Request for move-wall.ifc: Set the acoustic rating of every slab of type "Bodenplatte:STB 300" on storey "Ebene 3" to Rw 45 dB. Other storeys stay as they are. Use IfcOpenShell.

First a look at what the model holds.

```python
import ifcopenshell
import ifcopenshell.util.element

model = ifcopenshell.open("move-wall.ifc")
print(model.schema)
storey = next(s for s in model.by_type("IfcBuildingStorey") if s.Name == "Ebene 3")
slabs = [e for e in ifcopenshell.util.element.get_decomposition(storey) if e.is_a("IfcSlab")]
seen = {}
for e in slabs:
    element_type = ifcopenshell.util.element.get_type(e)
    key = (element_type.Name if element_type != e and element_type else None, ifcopenshell.util.element.get_pset(e, "Pset_SlabCommon", "AcousticRating"))
    seen[key] = seen.get(key, 0) + 1
for (name, value), count in sorted(seen.items(), key=str):
    print(count, "x", name, "|", value)
```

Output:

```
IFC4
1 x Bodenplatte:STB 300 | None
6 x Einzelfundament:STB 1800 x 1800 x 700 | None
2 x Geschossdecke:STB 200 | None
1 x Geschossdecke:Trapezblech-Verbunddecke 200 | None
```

```python
import ifcopenshell
import ifcopenshell.api.pset
import ifcopenshell.util.element

model = ifcopenshell.open("move-wall.ifc")

storey = next(s for s in model.by_type("IfcBuildingStorey") if s.Name == "Ebene 3")
slabs = [e for e in ifcopenshell.util.element.get_decomposition(storey) if e.is_a("IfcSlab")]

count = 0
for e in slabs:
    element_type = ifcopenshell.util.element.get_type(e)
    if element_type in (None, e) or element_type.Name != "Bodenplatte:STB 300":
        continue
    # add_pset returns the element's existing set when there is one.
    pset = ifcopenshell.api.pset.add_pset(model, product=e, name="Pset_SlabCommon")
    ifcopenshell.api.pset.edit_pset(model, pset=pset, properties={"AcousticRating": "Rw 45 dB"})
    count += 1

print(count, "slabs updated")

model.write("move-wall_updated.ifc")
```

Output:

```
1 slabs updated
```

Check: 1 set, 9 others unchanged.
